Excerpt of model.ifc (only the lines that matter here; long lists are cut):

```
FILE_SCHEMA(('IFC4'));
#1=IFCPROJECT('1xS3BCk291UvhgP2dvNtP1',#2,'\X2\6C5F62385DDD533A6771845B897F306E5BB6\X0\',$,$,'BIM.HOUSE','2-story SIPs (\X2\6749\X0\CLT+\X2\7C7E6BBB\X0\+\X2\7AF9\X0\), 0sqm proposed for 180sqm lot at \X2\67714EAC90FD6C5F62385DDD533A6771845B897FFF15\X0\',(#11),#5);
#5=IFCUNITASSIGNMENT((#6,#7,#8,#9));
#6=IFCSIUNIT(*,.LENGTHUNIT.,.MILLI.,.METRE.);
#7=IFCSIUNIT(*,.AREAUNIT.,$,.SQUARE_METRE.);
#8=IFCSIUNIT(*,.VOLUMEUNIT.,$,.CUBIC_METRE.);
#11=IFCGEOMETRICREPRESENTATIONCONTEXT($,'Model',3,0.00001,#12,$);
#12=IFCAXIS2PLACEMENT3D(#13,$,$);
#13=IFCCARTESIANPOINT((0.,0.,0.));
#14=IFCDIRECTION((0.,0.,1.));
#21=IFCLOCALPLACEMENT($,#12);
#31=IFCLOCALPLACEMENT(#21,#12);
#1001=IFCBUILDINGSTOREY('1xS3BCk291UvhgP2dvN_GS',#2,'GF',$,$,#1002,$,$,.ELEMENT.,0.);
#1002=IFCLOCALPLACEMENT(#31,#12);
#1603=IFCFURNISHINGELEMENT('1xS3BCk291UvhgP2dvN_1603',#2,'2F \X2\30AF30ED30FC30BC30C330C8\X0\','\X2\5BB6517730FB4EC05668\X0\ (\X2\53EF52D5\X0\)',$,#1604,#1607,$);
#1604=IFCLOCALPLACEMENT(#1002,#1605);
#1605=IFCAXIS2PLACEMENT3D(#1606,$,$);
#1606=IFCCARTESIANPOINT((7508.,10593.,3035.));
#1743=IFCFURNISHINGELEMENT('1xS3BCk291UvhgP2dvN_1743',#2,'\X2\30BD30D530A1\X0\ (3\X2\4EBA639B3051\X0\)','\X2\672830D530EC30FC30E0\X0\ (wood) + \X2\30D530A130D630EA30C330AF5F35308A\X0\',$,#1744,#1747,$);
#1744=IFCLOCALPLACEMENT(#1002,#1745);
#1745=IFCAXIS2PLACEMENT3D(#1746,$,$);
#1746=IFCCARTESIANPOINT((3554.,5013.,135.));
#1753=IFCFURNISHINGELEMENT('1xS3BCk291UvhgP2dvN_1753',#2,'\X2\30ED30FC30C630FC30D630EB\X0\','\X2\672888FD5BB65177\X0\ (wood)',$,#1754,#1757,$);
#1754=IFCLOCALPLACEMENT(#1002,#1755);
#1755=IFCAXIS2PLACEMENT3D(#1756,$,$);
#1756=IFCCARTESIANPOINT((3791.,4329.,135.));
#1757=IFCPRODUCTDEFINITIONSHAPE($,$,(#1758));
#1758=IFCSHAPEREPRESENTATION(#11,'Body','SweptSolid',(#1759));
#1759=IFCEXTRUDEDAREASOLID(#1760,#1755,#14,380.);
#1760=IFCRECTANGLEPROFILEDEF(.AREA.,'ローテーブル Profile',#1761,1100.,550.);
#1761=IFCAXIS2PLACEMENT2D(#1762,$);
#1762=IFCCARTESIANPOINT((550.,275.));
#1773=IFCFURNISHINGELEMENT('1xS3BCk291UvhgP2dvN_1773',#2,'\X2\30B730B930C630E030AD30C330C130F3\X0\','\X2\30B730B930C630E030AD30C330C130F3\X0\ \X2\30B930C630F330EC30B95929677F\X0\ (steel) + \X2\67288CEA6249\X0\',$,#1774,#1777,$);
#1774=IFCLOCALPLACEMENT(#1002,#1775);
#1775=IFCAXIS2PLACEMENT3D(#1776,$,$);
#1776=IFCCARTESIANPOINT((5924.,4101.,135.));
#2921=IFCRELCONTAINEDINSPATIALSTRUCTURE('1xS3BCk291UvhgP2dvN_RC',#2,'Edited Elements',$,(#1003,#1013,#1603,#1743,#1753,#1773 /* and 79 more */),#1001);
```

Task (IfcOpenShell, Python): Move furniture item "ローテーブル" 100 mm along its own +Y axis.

```python
import ifcopenshell
import ifcopenshell.api.geometry
import ifcopenshell.util.placement
import ifcopenshell.util.unit

model = ifcopenshell.open("model.ifc")
unit_scale = ifcopenshell.util.unit.calculate_unit_scale(model)

item = model.by_guid("1xS3BCk291UvhgP2dvN_1753")
matrix = ifcopenshell.util.placement.get_local_placement(item.ObjectPlacement)
matrix[:3, 3] += matrix[:3, 1] * 0.1 / unit_scale
ifcopenshell.api.geometry.edit_object_placement(model, product=item, matrix=matrix, is_si=False)

print(ifcopenshell.util.placement.get_local_placement(item.ObjectPlacement).round(3) + 0.0)

model.write("model_edited.ifc")
```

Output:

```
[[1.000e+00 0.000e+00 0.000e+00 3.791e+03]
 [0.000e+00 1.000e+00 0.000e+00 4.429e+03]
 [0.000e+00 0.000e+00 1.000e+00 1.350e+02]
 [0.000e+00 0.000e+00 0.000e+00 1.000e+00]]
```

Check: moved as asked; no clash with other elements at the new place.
